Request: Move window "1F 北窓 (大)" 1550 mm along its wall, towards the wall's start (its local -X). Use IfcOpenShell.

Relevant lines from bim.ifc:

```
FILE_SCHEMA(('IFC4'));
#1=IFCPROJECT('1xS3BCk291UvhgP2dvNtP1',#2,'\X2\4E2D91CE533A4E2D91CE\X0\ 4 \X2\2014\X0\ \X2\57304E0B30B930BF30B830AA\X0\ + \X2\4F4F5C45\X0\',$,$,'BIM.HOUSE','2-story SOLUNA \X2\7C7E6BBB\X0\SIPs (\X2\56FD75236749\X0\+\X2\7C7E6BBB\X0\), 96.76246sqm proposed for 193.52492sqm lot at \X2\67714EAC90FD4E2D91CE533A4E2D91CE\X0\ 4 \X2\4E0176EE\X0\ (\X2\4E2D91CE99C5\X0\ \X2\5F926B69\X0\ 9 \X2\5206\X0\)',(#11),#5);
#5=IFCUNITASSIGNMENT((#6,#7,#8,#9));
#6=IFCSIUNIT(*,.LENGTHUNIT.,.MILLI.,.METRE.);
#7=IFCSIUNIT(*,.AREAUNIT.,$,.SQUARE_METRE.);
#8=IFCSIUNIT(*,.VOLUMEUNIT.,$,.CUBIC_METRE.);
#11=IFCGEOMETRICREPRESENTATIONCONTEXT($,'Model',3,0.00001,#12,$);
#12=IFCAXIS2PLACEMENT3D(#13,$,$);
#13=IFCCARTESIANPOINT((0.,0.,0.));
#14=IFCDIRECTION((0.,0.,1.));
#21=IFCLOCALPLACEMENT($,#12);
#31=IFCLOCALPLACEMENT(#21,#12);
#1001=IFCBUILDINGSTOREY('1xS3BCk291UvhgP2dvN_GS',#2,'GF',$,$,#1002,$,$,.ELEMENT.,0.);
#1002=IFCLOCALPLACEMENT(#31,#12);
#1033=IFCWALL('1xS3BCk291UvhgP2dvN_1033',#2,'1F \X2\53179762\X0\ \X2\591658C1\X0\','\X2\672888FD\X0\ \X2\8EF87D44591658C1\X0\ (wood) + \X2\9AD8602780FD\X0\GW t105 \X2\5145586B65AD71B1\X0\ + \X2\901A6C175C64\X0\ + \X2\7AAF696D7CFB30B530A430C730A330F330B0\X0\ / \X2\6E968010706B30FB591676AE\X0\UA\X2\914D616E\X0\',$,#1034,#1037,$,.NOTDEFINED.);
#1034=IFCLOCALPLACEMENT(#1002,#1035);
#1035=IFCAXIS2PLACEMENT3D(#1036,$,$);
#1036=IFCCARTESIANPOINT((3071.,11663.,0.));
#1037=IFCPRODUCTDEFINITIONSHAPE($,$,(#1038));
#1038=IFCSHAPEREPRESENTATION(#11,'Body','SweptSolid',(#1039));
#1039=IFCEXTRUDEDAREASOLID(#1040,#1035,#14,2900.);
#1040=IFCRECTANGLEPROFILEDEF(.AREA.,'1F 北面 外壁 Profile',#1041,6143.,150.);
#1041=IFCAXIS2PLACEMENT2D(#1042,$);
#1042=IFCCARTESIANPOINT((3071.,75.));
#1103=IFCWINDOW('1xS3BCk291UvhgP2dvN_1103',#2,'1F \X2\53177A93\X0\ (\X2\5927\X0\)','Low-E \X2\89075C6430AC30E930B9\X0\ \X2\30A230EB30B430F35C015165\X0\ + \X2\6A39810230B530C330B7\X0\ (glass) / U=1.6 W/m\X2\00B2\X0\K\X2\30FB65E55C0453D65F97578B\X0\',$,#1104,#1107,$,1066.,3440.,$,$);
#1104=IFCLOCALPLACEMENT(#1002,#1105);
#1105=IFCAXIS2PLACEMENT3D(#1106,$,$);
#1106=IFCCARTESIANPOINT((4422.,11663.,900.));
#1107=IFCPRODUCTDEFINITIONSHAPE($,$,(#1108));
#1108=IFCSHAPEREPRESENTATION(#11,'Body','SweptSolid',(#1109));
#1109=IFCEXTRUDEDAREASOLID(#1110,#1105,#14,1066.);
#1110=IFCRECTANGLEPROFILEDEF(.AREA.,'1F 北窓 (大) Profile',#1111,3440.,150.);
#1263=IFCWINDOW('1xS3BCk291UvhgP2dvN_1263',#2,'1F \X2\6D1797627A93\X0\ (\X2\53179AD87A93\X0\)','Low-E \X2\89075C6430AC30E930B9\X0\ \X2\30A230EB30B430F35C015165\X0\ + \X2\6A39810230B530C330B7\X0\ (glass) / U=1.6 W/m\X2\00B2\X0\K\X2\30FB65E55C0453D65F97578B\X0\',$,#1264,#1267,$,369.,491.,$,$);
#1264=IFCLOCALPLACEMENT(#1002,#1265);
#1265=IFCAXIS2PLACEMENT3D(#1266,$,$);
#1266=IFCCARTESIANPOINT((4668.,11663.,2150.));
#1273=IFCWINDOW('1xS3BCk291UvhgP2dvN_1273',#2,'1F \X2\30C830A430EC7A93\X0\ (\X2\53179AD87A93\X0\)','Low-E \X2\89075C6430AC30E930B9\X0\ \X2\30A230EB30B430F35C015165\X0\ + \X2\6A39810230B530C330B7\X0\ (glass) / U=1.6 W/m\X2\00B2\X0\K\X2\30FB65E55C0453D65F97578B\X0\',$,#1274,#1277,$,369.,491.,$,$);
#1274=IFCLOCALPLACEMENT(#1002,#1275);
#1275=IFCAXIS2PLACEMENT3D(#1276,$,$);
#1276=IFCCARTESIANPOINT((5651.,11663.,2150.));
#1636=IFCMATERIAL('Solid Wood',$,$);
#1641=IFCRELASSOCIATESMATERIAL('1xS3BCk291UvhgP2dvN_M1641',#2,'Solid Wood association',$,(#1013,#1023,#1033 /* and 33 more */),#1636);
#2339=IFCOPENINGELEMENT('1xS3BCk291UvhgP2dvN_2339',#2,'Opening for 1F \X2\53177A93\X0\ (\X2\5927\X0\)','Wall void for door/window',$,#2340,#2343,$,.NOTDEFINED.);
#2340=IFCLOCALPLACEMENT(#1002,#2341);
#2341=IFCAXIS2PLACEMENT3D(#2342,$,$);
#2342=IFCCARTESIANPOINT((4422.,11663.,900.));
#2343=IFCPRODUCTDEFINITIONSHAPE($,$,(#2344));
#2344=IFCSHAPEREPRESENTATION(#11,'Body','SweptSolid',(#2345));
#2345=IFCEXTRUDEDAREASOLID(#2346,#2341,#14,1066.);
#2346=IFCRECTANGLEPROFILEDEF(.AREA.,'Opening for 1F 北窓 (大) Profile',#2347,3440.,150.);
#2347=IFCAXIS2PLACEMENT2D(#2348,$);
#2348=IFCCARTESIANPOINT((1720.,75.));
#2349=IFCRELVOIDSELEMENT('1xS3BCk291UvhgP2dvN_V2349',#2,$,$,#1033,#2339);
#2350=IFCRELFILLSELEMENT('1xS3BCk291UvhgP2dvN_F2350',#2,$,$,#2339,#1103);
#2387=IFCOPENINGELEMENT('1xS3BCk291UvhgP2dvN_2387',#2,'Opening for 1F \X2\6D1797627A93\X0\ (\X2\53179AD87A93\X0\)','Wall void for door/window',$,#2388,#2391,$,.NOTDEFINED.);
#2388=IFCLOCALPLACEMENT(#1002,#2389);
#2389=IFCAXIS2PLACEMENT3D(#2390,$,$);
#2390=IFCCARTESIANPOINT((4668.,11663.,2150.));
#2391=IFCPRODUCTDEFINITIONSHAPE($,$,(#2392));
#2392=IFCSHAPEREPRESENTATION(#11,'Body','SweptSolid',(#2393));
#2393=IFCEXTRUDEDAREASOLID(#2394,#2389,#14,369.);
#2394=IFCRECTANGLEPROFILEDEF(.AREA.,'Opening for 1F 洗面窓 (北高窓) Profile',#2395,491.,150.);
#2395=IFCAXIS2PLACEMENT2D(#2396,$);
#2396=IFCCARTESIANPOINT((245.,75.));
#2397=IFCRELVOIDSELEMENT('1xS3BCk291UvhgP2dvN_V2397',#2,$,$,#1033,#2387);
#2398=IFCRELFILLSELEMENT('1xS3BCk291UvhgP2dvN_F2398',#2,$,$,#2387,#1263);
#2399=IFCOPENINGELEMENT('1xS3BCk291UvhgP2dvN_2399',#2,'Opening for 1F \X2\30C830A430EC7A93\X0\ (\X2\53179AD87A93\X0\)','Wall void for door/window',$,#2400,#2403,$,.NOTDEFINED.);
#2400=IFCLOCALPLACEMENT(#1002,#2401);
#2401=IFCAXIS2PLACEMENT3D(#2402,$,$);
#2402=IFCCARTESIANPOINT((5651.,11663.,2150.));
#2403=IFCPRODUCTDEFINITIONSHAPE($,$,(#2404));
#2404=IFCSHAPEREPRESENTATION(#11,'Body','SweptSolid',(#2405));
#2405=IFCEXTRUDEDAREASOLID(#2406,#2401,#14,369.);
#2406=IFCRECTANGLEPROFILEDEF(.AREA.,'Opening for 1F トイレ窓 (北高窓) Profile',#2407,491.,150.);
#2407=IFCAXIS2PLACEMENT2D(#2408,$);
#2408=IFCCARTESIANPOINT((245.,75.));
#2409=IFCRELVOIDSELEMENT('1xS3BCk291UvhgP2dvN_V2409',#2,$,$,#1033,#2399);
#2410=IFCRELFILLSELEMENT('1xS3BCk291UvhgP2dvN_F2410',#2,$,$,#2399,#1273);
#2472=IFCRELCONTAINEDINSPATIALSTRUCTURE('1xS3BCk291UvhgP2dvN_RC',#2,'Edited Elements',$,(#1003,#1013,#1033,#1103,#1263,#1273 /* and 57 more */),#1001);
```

```python
import ifcopenshell
import ifcopenshell.api.geometry
import ifcopenshell.util.placement
import ifcopenshell.util.unit

model = ifcopenshell.open("bim.ifc")
unit_scale = ifcopenshell.util.unit.calculate_unit_scale(model)

window = model.by_guid("1xS3BCk291UvhgP2dvN_1103")
opening = window.FillsVoids[0].RelatingOpeningElement
wall = opening.VoidsElements[0].RelatingBuildingElement

wall_matrix = ifcopenshell.util.placement.get_local_placement(wall.ObjectPlacement)
shift = wall_matrix[:3, 0] * -1.55 / unit_scale
before = ifcopenshell.util.placement.get_local_placement(window.ObjectPlacement)[:3, 3].copy()

# The window is not placed relative to its opening, so move both.
for product in (opening, window):
    matrix = ifcopenshell.util.placement.get_local_placement(product.ObjectPlacement)
    matrix[:3, 3] += shift
    ifcopenshell.api.geometry.edit_object_placement(model, product=product, matrix=matrix, is_si=False)

after = ifcopenshell.util.placement.get_local_placement(window.ObjectPlacement)[:3, 3]
print("window moved by", (after - before).round(3) + 0.0)

model.write("bim_updated.ifc")
```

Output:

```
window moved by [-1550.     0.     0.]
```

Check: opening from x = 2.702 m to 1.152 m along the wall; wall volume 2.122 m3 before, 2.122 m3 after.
